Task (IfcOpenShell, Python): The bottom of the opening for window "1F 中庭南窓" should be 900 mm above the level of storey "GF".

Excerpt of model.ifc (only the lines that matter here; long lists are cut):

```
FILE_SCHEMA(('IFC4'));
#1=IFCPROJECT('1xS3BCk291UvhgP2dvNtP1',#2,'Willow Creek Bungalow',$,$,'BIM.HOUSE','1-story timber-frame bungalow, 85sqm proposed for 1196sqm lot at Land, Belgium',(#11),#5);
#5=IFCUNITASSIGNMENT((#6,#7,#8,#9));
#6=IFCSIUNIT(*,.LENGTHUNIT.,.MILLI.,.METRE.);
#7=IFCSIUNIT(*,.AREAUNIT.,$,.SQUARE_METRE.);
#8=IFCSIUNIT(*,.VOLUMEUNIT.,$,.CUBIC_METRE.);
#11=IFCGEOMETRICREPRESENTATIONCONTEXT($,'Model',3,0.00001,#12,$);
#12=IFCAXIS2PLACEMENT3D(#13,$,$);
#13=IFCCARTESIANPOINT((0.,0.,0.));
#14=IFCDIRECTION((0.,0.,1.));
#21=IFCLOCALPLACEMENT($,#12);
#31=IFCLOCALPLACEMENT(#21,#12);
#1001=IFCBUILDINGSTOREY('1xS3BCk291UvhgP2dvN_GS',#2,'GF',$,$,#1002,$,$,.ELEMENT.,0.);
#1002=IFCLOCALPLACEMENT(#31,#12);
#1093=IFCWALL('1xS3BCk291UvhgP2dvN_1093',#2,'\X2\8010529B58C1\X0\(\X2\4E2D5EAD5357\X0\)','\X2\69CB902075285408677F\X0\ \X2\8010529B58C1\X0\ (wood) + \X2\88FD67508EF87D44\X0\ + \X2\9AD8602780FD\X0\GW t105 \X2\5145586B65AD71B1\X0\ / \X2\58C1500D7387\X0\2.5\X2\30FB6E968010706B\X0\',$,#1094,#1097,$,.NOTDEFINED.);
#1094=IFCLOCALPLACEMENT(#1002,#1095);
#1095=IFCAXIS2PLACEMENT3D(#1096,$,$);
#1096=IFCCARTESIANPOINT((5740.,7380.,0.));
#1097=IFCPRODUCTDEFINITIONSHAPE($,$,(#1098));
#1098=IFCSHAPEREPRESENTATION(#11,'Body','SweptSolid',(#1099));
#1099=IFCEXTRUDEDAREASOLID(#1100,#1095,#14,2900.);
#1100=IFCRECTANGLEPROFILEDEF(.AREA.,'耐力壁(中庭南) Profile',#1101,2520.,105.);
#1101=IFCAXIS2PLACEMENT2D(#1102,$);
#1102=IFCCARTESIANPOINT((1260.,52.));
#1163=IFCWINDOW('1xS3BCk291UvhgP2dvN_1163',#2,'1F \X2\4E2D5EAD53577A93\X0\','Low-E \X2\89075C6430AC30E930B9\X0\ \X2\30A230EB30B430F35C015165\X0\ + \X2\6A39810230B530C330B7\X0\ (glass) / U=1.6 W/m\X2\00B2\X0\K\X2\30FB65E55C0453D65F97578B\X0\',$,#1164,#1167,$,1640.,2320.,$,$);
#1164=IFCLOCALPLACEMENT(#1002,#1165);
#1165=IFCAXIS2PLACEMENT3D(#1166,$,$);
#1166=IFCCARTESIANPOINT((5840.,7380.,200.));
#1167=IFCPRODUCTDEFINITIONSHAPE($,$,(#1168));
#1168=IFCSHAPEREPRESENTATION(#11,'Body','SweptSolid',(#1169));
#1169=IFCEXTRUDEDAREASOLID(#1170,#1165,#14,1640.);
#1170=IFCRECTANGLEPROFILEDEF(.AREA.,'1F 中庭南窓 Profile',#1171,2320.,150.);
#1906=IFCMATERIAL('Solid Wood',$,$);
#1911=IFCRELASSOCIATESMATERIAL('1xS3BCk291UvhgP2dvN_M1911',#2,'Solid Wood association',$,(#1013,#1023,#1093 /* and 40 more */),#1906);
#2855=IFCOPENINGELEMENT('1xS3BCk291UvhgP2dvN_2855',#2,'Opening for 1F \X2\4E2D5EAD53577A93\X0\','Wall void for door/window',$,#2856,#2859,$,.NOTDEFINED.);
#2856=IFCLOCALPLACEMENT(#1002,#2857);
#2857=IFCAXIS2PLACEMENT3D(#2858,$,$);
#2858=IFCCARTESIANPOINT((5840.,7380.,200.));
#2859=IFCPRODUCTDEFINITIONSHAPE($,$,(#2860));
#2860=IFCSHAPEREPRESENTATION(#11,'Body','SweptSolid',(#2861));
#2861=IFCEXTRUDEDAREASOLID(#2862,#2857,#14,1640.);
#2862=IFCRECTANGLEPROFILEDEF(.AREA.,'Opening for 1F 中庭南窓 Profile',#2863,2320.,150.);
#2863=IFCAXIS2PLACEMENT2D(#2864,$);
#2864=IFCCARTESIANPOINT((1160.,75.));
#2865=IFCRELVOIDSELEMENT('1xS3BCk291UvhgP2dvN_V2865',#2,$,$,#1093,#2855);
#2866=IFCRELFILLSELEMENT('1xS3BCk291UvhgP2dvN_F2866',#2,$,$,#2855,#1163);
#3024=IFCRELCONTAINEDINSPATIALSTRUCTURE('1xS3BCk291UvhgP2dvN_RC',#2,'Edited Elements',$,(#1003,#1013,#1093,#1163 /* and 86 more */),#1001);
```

```python
import numpy as np
import ifcopenshell
import ifcopenshell.api.geometry
import ifcopenshell.geom
import ifcopenshell.util.element
import ifcopenshell.util.placement
import ifcopenshell.util.shape
import ifcopenshell.util.unit

model = ifcopenshell.open("model.ifc")
unit_scale = ifcopenshell.util.unit.calculate_unit_scale(model)

window = model.by_guid("1xS3BCk291UvhgP2dvN_1163")
opening = window.FillsVoids[0].RelatingOpeningElement
storey = ifcopenshell.util.element.get_container(window, ifc_class="IfcBuildingStorey")
level = ifcopenshell.util.placement.get_local_placement(storey.ObjectPlacement)[2, 3]

# The opening's origin need not be at the sill, so measure its lowest point.
shape = ifcopenshell.geom.create_shape(ifcopenshell.geom.settings(), opening)
bottom = ifcopenshell.util.shape.get_shape_bottom_elevation(shape, shape.geometry) / unit_scale
dz = level + 0.9 / unit_scale - bottom

shift = np.array([0.0, 0.0, dz])
# The window is not placed relative to its opening, so move both.
for product in (opening, window):
    matrix = ifcopenshell.util.placement.get_local_placement(product.ObjectPlacement)
    matrix[:3, 3] += shift
    ifcopenshell.api.geometry.edit_object_placement(model, product=product, matrix=matrix, is_si=False)

print(f"moved by {dz * unit_scale:+.3f} m")

model.write("model_edited.ifc")
```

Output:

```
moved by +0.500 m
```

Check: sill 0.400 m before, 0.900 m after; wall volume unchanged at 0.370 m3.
